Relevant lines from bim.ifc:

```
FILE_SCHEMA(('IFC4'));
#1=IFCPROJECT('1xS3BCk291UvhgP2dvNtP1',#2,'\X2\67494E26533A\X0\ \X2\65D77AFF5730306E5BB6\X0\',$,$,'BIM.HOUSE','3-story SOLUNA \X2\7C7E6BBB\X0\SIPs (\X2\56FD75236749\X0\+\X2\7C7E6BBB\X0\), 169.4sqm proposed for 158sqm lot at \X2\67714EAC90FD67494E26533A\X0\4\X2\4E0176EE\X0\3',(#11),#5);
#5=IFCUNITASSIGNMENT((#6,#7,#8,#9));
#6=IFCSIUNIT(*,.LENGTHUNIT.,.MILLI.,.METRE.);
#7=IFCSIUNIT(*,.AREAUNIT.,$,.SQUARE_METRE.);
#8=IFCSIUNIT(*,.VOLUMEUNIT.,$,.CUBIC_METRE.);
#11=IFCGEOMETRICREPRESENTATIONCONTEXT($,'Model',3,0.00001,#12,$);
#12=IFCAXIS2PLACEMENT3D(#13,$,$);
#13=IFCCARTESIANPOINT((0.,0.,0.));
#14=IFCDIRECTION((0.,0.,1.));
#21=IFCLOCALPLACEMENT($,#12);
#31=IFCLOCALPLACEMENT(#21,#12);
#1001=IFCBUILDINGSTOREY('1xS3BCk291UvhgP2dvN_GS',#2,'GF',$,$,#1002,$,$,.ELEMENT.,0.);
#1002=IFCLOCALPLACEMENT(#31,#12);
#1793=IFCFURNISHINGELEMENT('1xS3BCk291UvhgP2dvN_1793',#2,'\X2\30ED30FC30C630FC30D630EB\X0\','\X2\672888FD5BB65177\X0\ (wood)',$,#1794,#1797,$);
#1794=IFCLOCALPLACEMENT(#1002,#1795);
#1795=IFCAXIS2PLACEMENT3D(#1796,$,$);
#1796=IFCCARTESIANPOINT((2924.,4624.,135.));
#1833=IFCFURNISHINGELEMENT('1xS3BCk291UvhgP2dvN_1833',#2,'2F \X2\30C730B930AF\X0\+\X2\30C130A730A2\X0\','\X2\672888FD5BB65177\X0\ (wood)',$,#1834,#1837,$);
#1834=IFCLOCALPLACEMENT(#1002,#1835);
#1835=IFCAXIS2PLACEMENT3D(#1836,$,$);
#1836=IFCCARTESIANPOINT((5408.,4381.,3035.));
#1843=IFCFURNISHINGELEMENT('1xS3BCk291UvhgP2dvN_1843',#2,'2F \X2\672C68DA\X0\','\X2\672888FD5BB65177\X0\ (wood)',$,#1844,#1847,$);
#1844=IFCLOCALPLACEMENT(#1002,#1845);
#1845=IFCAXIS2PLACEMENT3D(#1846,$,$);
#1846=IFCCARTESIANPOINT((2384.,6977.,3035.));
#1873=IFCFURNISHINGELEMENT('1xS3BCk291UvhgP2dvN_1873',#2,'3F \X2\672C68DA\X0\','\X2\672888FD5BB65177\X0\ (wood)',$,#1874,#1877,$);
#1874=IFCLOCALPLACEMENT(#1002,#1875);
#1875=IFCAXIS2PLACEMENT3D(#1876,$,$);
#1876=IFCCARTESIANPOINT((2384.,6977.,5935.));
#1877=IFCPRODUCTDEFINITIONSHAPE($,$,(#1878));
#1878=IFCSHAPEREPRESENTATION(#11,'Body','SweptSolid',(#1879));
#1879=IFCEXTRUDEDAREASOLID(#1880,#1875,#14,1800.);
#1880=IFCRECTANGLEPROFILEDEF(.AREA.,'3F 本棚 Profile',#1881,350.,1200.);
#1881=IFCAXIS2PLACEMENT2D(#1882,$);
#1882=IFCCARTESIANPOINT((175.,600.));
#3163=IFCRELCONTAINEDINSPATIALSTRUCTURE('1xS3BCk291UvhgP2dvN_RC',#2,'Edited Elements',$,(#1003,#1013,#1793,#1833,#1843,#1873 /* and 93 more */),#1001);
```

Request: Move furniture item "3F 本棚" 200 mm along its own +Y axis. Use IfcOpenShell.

```python
import ifcopenshell
import ifcopenshell.api.geometry
import ifcopenshell.util.placement
import ifcopenshell.util.unit

model = ifcopenshell.open("bim.ifc")
unit_scale = ifcopenshell.util.unit.calculate_unit_scale(model)

item = model.by_id(1873)
matrix = ifcopenshell.util.placement.get_local_placement(item.ObjectPlacement)
matrix[:3, 3] += matrix[:3, 1] * 0.2 / unit_scale
ifcopenshell.api.geometry.edit_object_placement(model, product=item, matrix=matrix, is_si=False)

print(ifcopenshell.util.placement.get_local_placement(item.ObjectPlacement).round(3) + 0.0)

model.write("bim_edited.ifc")
```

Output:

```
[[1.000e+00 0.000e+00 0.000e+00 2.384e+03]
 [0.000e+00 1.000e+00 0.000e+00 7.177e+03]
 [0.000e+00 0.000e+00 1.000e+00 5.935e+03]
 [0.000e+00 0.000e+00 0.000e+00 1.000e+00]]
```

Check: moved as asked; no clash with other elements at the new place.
